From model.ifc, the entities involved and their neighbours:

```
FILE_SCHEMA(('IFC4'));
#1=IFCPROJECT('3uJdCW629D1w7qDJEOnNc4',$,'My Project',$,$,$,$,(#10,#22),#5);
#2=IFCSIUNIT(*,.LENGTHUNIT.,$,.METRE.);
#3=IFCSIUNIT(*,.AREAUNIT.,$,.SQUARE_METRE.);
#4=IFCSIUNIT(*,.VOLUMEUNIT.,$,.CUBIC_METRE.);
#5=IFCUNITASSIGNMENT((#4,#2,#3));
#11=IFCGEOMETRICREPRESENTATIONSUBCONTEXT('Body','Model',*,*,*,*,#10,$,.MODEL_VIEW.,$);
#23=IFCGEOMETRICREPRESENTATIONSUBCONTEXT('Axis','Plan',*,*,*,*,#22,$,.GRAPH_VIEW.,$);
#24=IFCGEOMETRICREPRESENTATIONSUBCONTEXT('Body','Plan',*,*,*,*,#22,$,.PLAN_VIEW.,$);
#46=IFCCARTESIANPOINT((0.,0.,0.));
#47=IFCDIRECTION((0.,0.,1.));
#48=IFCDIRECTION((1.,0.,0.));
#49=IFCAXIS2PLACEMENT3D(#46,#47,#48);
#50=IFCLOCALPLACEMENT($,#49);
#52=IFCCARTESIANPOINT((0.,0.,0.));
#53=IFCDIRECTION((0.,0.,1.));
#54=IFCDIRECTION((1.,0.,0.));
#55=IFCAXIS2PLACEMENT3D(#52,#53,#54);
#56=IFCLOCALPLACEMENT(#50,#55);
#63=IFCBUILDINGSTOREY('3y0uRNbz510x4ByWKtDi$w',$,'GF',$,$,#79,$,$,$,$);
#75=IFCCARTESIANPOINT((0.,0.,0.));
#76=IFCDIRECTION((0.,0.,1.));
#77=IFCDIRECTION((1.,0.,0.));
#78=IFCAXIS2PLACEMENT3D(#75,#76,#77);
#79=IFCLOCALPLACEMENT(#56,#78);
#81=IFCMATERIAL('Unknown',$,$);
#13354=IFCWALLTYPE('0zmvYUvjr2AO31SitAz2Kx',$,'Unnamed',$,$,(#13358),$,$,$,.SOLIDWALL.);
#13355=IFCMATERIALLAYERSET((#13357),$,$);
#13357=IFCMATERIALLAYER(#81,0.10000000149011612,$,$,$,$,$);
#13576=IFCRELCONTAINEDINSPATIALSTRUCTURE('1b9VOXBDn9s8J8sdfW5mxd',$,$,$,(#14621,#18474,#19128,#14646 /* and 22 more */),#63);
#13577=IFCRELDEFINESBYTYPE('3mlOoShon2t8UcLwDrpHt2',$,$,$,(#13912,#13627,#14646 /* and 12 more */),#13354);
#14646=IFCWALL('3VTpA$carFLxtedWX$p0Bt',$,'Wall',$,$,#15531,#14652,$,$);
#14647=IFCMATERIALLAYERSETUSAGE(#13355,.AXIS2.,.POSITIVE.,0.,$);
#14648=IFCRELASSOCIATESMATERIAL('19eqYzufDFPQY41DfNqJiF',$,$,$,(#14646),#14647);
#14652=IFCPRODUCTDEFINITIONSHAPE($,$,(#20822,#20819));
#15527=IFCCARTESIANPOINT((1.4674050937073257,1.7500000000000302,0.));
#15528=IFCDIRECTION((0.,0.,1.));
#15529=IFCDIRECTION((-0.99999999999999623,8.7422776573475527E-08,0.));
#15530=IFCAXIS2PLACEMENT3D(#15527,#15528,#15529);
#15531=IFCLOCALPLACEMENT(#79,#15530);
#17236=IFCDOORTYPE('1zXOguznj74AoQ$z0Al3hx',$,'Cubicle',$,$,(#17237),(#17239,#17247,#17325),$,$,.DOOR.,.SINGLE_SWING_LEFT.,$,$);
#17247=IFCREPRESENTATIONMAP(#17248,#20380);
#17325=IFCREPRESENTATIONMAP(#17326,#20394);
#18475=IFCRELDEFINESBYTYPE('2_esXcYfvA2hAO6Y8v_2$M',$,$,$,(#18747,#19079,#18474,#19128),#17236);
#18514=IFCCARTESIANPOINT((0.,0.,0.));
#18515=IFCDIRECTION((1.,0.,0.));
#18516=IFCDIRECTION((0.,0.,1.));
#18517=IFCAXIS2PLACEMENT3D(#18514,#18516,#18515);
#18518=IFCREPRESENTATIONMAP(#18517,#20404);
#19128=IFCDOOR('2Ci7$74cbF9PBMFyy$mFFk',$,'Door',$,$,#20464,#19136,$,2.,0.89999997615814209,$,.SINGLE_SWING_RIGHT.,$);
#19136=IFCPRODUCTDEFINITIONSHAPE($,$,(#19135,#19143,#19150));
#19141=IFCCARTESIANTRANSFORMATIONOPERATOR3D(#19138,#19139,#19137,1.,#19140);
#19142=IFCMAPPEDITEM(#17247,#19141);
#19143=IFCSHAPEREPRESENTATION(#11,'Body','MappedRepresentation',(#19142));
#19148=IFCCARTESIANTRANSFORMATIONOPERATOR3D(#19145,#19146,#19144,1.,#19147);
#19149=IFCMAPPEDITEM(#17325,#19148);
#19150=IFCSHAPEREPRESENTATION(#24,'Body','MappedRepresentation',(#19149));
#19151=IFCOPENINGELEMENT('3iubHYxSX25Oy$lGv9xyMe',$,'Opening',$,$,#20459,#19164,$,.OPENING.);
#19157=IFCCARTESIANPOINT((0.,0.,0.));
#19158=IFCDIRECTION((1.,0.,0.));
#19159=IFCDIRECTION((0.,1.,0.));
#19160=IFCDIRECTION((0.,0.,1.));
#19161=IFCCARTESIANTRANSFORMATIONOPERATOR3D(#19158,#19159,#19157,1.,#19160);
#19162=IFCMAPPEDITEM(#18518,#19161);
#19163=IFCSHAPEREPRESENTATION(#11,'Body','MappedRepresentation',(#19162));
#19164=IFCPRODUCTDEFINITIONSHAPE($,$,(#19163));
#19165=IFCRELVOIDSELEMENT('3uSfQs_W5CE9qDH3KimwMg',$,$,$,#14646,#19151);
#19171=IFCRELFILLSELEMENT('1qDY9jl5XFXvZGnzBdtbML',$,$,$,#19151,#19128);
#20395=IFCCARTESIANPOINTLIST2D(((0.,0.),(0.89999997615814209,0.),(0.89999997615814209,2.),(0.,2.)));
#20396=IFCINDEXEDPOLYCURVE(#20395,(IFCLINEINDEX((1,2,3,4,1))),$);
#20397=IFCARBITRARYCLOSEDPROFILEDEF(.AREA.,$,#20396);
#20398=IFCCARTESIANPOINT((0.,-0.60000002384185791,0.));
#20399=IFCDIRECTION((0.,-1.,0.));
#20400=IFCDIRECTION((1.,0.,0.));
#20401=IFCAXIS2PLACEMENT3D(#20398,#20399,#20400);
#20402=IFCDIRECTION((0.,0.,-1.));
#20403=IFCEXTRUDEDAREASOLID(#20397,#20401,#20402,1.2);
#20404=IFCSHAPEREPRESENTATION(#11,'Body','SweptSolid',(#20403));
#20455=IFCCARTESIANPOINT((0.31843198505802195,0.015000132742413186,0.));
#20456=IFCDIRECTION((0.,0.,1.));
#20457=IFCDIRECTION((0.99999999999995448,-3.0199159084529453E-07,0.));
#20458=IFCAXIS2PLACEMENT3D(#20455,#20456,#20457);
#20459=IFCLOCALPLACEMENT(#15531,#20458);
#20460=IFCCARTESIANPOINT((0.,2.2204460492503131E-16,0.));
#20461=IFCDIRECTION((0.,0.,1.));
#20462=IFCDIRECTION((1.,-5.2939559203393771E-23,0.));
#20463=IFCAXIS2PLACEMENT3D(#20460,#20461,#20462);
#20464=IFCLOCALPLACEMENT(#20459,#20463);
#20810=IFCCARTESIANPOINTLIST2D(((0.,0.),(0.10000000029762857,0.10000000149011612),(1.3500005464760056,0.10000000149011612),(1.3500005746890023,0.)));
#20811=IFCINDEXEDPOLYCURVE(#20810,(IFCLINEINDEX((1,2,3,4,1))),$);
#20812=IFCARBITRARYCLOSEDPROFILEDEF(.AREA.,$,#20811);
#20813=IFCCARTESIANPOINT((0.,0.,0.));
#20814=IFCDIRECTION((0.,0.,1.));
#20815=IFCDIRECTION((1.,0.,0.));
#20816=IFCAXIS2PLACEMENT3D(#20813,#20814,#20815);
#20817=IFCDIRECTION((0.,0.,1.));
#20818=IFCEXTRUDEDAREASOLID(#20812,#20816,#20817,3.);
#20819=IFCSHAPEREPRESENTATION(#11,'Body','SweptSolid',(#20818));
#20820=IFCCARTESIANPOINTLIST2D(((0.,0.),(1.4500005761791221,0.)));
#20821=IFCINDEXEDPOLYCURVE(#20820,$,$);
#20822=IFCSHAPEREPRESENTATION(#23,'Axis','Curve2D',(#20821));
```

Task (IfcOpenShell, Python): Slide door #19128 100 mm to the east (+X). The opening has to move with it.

```python
import ifcopenshell
import ifcopenshell.api.geometry
import ifcopenshell.util.placement
import ifcopenshell.util.unit

model = ifcopenshell.open("model.ifc")
unit_scale = ifcopenshell.util.unit.calculate_unit_scale(model)

door = model.by_guid("2Ci7$74cbF9PBMFyy$mFFk")
opening = door.FillsVoids[0].RelatingOpeningElement
wall = opening.VoidsElements[0].RelatingBuildingElement

wall_matrix = ifcopenshell.util.placement.get_local_placement(wall.ObjectPlacement)
shift = wall_matrix[:3, 0] * -0.1 / unit_scale
before = ifcopenshell.util.placement.get_local_placement(door.ObjectPlacement)[:3, 3].copy()

# The door is placed relative to its opening, so it follows when the opening moves.
matrix = ifcopenshell.util.placement.get_local_placement(opening.ObjectPlacement)
matrix[:3, 3] += shift
ifcopenshell.api.geometry.edit_object_placement(
    model, product=opening, matrix=matrix, is_si=False, should_transform_children=True
)

after = ifcopenshell.util.placement.get_local_placement(door.ObjectPlacement)[:3, 3]
print("door moved by", (after - before).round(3) + 0.0)

model.write("model-out.ifc")
```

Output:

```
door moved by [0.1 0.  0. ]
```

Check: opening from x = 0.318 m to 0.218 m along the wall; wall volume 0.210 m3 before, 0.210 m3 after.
